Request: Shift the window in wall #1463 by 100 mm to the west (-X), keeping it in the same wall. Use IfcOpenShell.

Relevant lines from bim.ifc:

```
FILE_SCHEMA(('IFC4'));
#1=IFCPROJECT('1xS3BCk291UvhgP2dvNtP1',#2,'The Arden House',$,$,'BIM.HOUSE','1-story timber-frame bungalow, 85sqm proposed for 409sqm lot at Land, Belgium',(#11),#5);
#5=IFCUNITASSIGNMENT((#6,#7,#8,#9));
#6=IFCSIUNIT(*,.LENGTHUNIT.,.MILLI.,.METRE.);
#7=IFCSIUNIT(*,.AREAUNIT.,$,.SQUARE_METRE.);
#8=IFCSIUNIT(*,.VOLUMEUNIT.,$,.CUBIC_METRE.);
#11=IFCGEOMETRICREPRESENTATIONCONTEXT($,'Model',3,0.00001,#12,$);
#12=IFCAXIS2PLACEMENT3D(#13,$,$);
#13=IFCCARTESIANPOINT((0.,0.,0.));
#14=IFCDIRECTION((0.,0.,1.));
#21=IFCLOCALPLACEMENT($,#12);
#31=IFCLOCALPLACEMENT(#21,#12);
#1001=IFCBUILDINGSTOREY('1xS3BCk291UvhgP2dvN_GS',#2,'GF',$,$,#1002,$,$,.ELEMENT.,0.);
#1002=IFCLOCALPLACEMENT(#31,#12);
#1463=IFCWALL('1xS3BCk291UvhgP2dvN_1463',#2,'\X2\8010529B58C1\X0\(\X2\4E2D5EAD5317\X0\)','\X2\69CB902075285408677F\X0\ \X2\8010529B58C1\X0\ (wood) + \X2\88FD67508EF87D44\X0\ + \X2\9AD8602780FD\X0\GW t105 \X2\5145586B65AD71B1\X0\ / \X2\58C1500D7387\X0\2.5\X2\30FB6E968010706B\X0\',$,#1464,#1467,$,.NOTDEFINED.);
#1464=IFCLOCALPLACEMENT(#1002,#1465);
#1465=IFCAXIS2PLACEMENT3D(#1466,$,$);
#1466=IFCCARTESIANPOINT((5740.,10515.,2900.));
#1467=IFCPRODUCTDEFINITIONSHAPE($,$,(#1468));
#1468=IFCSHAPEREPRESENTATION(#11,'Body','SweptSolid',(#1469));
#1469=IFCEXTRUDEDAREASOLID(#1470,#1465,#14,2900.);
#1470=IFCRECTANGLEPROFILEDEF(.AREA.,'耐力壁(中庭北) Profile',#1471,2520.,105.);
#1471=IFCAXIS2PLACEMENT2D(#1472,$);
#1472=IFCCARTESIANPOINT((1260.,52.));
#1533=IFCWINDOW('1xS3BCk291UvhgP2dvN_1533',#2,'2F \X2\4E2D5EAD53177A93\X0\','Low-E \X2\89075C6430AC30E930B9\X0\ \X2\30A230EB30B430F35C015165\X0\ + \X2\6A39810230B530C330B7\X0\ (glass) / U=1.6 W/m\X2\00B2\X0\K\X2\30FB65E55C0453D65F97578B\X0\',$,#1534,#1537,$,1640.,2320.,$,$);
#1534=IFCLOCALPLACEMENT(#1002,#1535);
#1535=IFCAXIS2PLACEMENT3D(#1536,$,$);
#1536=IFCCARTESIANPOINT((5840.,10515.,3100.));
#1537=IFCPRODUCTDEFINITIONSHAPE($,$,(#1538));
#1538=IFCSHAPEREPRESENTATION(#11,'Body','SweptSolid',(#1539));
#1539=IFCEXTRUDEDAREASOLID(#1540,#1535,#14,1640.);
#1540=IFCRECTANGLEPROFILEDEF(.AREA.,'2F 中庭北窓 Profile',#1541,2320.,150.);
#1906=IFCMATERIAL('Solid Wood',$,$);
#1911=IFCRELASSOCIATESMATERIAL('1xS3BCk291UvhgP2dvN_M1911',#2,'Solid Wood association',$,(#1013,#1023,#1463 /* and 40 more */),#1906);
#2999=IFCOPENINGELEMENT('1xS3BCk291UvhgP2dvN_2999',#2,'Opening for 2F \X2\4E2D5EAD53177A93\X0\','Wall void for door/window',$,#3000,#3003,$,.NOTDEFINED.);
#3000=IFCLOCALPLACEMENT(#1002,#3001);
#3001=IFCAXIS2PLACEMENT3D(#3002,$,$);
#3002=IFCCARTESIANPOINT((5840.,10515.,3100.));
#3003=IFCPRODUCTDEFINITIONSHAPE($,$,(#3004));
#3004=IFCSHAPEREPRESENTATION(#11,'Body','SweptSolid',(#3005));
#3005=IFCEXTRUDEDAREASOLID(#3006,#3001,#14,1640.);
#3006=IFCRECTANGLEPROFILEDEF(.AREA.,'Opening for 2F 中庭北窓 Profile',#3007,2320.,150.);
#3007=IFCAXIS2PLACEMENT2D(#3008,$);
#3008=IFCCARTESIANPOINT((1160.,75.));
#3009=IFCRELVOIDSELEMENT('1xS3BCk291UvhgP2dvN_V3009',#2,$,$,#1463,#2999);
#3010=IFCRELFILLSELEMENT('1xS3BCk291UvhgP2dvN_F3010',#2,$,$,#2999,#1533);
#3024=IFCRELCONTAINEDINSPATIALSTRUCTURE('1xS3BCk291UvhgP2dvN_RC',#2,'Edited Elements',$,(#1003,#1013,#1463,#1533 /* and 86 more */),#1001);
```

```python
import ifcopenshell
import ifcopenshell.api.geometry
import ifcopenshell.util.placement

model = ifcopenshell.open("bim.ifc")

window = model.by_guid("1xS3BCk291UvhgP2dvN_1533")
opening = window.FillsVoids[0].RelatingOpeningElement
wall = opening.VoidsElements[0].RelatingBuildingElement

wall_matrix = ifcopenshell.util.placement.get_local_placement(wall.ObjectPlacement)
shift = wall_matrix[:3, 0] * -100.0
before = ifcopenshell.util.placement.get_local_placement(window.ObjectPlacement)[:3, 3].copy()

# The window is not placed relative to its opening, so move both.
for product in (opening, window):
    matrix = ifcopenshell.util.placement.get_local_placement(product.ObjectPlacement)
    matrix[:3, 3] += shift
    ifcopenshell.api.geometry.edit_object_placement(model, product=product, matrix=matrix, is_si=False)

after = ifcopenshell.util.placement.get_local_placement(window.ObjectPlacement)[:3, 3]
print("window moved by", (after - before).round(3) + 0.0)

model.write("bim-out.ifc")
```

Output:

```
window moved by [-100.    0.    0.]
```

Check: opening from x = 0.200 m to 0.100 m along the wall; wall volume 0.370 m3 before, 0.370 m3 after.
